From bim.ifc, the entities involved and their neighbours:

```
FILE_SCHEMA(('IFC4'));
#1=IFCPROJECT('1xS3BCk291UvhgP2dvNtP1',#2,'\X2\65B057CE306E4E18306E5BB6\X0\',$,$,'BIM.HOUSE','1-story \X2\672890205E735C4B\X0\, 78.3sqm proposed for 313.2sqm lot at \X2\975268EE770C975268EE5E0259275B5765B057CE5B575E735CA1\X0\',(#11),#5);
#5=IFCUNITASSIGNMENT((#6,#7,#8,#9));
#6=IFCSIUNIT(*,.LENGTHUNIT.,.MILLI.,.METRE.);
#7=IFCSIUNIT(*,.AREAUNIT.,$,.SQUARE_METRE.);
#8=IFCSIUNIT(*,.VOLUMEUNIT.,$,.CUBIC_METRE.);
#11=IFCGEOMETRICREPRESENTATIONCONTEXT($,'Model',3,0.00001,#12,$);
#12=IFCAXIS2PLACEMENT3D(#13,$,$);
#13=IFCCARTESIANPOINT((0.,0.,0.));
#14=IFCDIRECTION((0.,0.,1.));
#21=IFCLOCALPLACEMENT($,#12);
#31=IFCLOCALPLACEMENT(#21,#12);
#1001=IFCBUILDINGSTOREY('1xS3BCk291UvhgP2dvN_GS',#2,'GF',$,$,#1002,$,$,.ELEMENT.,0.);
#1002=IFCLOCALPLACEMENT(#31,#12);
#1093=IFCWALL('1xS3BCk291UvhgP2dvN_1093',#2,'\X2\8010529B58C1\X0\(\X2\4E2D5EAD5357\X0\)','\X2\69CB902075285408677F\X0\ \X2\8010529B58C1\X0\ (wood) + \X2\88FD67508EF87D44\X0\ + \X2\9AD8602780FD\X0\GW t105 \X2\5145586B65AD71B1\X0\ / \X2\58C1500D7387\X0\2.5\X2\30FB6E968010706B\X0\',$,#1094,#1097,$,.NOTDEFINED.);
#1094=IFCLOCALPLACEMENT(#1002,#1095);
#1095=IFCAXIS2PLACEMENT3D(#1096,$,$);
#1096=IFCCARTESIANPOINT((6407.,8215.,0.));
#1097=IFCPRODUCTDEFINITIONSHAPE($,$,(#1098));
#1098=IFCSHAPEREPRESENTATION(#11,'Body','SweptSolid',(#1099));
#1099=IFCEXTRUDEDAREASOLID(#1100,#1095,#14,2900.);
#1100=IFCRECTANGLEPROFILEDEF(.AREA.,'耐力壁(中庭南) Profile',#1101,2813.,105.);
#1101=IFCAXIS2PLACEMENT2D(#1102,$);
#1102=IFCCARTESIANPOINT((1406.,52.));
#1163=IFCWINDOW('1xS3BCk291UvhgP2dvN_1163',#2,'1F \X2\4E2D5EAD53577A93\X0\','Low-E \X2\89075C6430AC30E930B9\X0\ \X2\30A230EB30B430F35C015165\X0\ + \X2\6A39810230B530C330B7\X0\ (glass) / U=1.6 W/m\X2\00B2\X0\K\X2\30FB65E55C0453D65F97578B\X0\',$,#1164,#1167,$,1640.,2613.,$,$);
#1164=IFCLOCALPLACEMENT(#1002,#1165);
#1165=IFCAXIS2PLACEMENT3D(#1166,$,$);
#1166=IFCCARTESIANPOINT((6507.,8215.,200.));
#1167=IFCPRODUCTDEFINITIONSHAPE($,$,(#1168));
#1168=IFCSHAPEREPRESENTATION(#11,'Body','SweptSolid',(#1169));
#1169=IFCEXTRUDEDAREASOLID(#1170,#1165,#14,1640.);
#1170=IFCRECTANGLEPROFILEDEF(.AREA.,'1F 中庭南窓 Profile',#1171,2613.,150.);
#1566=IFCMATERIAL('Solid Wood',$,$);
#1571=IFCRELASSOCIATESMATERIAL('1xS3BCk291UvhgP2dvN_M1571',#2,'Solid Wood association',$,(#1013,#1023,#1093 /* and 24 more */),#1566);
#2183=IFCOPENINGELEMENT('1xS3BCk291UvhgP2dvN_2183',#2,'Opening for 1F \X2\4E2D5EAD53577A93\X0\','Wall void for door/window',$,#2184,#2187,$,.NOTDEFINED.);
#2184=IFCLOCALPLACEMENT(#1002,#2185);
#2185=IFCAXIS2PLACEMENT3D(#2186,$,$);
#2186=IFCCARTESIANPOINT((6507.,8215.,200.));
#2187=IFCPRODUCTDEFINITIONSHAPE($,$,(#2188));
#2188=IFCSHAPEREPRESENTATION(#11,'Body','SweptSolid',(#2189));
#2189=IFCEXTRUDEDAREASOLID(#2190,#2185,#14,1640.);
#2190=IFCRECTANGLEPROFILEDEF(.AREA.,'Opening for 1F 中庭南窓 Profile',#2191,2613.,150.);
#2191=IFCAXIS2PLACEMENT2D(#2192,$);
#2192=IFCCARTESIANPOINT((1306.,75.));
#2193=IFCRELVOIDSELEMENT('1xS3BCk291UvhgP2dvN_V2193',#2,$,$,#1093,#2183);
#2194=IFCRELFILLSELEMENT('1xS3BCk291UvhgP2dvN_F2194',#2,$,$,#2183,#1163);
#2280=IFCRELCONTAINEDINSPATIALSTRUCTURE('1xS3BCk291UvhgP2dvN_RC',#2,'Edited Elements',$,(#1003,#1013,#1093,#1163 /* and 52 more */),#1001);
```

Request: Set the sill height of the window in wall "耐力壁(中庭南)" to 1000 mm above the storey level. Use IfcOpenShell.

```python
import numpy as np
import ifcopenshell
import ifcopenshell.api.geometry
import ifcopenshell.geom
import ifcopenshell.util.element
import ifcopenshell.util.placement
import ifcopenshell.util.shape
import ifcopenshell.util.unit

model = ifcopenshell.open("bim.ifc")
unit_scale = ifcopenshell.util.unit.calculate_unit_scale(model)

window = model.by_guid("1xS3BCk291UvhgP2dvN_1163")
opening = window.FillsVoids[0].RelatingOpeningElement
storey = ifcopenshell.util.element.get_container(window, ifc_class="IfcBuildingStorey")
level = ifcopenshell.util.placement.get_local_placement(storey.ObjectPlacement)[2, 3]

# The opening's origin need not be at the sill, so measure its lowest point.
shape = ifcopenshell.geom.create_shape(ifcopenshell.geom.settings(), opening)
bottom = ifcopenshell.util.shape.get_shape_bottom_elevation(shape, shape.geometry) / unit_scale
dz = level + 1 / unit_scale - bottom

shift = np.array([0.0, 0.0, dz])
# The window is not placed relative to its opening, so move both.
for product in (opening, window):
    matrix = ifcopenshell.util.placement.get_local_placement(product.ObjectPlacement)
    matrix[:3, 3] += shift
    ifcopenshell.api.geometry.edit_object_placement(model, product=product, matrix=matrix, is_si=False)

print(f"moved by {dz * unit_scale:+.3f} m")

model.write("bim_updated.ifc")
```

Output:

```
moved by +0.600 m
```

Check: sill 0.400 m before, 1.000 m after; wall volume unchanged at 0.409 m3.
